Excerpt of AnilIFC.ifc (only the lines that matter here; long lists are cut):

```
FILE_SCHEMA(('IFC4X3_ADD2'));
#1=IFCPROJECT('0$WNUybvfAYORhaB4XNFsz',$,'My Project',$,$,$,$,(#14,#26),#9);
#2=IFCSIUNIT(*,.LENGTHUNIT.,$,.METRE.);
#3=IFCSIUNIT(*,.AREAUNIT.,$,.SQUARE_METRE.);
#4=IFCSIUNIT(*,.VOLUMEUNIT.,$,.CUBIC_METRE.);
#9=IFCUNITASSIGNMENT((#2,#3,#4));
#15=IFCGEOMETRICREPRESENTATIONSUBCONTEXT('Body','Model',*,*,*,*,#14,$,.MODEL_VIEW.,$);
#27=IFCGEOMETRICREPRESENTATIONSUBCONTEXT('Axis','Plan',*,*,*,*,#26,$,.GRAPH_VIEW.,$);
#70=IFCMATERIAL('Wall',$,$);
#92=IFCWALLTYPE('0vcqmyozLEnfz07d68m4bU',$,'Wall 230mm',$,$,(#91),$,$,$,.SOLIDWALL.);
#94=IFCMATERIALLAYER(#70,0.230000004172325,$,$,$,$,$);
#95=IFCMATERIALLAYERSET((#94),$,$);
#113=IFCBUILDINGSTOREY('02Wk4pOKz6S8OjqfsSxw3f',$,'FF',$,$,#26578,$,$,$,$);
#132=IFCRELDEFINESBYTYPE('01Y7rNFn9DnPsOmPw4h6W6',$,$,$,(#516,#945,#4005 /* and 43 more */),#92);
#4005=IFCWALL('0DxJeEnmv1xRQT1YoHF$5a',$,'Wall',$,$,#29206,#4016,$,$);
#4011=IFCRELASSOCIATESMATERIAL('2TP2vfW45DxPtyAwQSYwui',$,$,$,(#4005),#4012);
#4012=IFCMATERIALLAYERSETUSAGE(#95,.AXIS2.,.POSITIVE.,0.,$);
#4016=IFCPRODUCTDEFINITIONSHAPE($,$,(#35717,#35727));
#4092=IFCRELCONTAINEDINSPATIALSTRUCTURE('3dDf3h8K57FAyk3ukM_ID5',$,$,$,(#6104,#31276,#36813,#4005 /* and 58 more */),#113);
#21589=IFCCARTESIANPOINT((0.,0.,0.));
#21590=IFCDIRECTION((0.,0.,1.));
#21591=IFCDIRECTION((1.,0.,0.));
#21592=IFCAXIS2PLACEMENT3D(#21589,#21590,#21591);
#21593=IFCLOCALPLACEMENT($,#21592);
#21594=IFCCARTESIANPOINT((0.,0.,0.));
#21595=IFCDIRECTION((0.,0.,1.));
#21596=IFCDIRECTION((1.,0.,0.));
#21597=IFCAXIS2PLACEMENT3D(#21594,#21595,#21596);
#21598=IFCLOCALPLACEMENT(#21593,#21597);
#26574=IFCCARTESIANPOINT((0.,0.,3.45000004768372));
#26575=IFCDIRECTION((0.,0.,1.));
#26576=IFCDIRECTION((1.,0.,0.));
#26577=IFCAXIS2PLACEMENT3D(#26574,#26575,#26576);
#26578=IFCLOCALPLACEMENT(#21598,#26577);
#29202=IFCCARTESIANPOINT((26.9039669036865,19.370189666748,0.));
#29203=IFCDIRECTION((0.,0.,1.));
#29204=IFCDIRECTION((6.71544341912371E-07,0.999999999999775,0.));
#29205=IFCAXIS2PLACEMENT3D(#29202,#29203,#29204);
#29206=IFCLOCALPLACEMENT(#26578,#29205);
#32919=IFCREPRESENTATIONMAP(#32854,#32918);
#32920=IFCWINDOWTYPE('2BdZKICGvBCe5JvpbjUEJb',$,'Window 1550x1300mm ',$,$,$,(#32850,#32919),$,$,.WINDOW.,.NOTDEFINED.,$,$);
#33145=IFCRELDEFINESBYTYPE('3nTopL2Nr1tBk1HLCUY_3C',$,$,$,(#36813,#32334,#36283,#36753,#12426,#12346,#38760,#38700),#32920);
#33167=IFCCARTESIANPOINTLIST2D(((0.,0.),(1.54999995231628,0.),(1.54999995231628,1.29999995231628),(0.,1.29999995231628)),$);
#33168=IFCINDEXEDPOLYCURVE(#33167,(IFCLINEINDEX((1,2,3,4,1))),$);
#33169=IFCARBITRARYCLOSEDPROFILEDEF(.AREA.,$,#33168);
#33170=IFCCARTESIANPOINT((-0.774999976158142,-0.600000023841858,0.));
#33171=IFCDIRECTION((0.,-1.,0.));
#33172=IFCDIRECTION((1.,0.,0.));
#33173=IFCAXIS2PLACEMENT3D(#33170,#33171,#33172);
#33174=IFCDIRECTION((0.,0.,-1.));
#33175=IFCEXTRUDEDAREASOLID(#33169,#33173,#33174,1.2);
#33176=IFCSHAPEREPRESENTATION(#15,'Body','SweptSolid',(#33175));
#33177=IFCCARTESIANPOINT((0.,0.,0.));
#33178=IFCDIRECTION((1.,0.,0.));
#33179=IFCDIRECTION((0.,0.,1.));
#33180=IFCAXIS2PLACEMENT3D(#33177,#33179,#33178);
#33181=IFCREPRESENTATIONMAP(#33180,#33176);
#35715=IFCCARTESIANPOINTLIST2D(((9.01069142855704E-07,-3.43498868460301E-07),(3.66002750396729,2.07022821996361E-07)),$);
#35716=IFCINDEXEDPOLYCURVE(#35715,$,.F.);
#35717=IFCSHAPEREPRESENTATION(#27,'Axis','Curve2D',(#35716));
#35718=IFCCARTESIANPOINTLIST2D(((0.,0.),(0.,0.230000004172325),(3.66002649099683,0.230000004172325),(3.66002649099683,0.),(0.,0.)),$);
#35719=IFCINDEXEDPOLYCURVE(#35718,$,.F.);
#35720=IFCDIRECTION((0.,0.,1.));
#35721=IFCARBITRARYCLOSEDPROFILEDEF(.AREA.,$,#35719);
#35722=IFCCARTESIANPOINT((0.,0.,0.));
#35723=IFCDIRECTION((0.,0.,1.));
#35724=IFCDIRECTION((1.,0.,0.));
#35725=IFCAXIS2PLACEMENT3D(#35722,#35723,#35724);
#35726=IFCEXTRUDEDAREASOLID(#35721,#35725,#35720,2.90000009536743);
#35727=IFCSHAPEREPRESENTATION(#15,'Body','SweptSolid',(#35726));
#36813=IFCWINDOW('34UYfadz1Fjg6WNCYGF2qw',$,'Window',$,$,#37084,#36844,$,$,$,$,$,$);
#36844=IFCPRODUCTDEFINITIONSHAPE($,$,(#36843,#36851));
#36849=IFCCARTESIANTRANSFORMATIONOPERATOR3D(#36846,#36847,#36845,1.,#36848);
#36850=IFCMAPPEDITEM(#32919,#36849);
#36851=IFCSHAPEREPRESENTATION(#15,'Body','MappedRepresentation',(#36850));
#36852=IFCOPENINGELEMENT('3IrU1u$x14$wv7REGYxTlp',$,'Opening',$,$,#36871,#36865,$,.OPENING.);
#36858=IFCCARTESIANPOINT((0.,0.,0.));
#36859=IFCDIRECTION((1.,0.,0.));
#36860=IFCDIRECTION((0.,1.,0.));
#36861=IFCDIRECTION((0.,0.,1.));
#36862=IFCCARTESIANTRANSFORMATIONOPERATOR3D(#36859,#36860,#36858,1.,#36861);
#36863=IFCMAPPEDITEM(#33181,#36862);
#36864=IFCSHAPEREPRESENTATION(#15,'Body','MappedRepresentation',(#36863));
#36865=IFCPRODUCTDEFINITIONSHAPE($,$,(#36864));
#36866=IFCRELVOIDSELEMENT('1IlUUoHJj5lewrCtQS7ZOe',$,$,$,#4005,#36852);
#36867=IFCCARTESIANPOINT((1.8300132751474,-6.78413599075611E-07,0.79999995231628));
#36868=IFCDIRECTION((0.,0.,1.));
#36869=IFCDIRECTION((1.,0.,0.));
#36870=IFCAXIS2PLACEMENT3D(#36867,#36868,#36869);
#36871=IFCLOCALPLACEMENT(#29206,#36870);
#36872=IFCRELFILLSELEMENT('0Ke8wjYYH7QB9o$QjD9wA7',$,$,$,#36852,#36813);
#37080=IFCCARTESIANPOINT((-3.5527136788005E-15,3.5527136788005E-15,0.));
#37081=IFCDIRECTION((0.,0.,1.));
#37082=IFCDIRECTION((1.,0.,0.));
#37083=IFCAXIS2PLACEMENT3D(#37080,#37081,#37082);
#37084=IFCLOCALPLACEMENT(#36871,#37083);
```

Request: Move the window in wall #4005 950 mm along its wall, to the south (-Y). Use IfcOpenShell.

```python
import ifcopenshell
import ifcopenshell.api.geometry
import ifcopenshell.util.placement

model = ifcopenshell.open("AnilIFC.ifc")

window = model.by_guid("34UYfadz1Fjg6WNCYGF2qw")
opening = window.FillsVoids[0].RelatingOpeningElement
wall = opening.VoidsElements[0].RelatingBuildingElement

wall_matrix = ifcopenshell.util.placement.get_local_placement(wall.ObjectPlacement)
shift = wall_matrix[:3, 0] * -0.95
before = ifcopenshell.util.placement.get_local_placement(window.ObjectPlacement)[:3, 3].copy()

# The window is placed relative to its opening, so it follows when the opening moves.
matrix = ifcopenshell.util.placement.get_local_placement(opening.ObjectPlacement)
matrix[:3, 3] += shift
ifcopenshell.api.geometry.edit_object_placement(
    model, product=opening, matrix=matrix, is_si=False, should_transform_children=True
)

after = ifcopenshell.util.placement.get_local_placement(window.ObjectPlacement)[:3, 3]
print("window moved by", (after - before).round(3) + 0.0)

model.write("AnilIFC_updated.ifc")
```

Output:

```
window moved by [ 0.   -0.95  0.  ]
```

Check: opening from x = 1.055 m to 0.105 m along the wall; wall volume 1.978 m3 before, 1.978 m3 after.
